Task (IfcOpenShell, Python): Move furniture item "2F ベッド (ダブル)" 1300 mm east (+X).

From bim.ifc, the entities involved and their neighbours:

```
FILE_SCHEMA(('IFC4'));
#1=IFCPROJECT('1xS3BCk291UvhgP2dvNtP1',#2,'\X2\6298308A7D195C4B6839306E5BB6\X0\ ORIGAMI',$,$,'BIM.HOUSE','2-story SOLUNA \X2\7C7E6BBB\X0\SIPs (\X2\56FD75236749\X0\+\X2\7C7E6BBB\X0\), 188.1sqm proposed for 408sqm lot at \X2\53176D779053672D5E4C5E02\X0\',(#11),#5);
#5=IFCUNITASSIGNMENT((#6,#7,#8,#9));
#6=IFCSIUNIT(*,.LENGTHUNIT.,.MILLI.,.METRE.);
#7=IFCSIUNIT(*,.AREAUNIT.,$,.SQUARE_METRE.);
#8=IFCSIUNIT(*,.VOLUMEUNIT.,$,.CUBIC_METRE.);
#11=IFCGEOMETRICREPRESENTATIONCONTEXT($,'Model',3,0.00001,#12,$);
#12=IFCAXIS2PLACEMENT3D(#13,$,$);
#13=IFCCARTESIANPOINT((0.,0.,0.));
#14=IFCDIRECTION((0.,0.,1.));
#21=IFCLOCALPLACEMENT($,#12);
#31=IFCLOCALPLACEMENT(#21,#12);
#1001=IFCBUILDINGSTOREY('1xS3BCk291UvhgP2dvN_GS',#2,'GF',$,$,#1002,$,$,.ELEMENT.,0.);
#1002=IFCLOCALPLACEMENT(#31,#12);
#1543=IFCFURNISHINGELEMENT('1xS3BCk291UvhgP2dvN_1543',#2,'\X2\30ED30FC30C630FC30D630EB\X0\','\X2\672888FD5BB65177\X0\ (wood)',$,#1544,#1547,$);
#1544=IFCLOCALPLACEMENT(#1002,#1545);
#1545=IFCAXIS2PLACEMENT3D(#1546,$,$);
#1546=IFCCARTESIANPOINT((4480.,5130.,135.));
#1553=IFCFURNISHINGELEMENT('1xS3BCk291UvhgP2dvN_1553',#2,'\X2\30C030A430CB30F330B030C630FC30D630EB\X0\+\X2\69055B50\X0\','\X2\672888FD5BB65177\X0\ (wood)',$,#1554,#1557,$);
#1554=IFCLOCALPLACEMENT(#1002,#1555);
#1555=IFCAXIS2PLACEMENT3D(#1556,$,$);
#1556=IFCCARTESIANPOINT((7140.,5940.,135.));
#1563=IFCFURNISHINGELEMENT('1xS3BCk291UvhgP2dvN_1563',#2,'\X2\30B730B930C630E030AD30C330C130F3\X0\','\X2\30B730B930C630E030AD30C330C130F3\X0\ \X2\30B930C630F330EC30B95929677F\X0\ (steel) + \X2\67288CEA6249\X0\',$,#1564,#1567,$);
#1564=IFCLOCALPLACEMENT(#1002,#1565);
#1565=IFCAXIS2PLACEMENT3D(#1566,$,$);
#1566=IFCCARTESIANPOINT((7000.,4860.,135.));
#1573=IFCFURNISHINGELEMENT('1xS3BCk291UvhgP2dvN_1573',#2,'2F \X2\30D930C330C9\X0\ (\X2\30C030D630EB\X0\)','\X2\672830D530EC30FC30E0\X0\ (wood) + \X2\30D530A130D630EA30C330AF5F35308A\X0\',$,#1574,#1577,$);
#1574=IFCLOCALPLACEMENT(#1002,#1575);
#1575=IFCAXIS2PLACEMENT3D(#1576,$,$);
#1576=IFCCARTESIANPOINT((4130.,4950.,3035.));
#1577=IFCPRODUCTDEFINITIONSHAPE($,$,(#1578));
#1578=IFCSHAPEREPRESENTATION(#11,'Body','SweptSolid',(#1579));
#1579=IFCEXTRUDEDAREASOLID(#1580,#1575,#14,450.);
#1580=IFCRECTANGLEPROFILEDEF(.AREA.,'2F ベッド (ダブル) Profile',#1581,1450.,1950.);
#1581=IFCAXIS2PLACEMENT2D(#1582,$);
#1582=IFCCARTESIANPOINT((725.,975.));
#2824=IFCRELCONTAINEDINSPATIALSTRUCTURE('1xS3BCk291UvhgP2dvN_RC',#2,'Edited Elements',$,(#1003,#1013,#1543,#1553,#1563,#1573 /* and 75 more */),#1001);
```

```python
import ifcopenshell
import ifcopenshell.api.geometry
import ifcopenshell.util.placement
import ifcopenshell.util.unit

model = ifcopenshell.open("bim.ifc")
unit_scale = ifcopenshell.util.unit.calculate_unit_scale(model)

item = model.by_guid("1xS3BCk291UvhgP2dvN_1573")
matrix = ifcopenshell.util.placement.get_local_placement(item.ObjectPlacement)
matrix[0, 3] += 1.3 / unit_scale
ifcopenshell.api.geometry.edit_object_placement(model, product=item, matrix=matrix, is_si=False)

print(ifcopenshell.util.placement.get_local_placement(item.ObjectPlacement).round(3) + 0.0)

model.write("bim_edited.ifc")
```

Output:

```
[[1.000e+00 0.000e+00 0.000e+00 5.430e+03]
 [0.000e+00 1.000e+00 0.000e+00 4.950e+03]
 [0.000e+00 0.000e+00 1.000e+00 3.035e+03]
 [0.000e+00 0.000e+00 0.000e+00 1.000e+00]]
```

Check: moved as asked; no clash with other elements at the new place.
